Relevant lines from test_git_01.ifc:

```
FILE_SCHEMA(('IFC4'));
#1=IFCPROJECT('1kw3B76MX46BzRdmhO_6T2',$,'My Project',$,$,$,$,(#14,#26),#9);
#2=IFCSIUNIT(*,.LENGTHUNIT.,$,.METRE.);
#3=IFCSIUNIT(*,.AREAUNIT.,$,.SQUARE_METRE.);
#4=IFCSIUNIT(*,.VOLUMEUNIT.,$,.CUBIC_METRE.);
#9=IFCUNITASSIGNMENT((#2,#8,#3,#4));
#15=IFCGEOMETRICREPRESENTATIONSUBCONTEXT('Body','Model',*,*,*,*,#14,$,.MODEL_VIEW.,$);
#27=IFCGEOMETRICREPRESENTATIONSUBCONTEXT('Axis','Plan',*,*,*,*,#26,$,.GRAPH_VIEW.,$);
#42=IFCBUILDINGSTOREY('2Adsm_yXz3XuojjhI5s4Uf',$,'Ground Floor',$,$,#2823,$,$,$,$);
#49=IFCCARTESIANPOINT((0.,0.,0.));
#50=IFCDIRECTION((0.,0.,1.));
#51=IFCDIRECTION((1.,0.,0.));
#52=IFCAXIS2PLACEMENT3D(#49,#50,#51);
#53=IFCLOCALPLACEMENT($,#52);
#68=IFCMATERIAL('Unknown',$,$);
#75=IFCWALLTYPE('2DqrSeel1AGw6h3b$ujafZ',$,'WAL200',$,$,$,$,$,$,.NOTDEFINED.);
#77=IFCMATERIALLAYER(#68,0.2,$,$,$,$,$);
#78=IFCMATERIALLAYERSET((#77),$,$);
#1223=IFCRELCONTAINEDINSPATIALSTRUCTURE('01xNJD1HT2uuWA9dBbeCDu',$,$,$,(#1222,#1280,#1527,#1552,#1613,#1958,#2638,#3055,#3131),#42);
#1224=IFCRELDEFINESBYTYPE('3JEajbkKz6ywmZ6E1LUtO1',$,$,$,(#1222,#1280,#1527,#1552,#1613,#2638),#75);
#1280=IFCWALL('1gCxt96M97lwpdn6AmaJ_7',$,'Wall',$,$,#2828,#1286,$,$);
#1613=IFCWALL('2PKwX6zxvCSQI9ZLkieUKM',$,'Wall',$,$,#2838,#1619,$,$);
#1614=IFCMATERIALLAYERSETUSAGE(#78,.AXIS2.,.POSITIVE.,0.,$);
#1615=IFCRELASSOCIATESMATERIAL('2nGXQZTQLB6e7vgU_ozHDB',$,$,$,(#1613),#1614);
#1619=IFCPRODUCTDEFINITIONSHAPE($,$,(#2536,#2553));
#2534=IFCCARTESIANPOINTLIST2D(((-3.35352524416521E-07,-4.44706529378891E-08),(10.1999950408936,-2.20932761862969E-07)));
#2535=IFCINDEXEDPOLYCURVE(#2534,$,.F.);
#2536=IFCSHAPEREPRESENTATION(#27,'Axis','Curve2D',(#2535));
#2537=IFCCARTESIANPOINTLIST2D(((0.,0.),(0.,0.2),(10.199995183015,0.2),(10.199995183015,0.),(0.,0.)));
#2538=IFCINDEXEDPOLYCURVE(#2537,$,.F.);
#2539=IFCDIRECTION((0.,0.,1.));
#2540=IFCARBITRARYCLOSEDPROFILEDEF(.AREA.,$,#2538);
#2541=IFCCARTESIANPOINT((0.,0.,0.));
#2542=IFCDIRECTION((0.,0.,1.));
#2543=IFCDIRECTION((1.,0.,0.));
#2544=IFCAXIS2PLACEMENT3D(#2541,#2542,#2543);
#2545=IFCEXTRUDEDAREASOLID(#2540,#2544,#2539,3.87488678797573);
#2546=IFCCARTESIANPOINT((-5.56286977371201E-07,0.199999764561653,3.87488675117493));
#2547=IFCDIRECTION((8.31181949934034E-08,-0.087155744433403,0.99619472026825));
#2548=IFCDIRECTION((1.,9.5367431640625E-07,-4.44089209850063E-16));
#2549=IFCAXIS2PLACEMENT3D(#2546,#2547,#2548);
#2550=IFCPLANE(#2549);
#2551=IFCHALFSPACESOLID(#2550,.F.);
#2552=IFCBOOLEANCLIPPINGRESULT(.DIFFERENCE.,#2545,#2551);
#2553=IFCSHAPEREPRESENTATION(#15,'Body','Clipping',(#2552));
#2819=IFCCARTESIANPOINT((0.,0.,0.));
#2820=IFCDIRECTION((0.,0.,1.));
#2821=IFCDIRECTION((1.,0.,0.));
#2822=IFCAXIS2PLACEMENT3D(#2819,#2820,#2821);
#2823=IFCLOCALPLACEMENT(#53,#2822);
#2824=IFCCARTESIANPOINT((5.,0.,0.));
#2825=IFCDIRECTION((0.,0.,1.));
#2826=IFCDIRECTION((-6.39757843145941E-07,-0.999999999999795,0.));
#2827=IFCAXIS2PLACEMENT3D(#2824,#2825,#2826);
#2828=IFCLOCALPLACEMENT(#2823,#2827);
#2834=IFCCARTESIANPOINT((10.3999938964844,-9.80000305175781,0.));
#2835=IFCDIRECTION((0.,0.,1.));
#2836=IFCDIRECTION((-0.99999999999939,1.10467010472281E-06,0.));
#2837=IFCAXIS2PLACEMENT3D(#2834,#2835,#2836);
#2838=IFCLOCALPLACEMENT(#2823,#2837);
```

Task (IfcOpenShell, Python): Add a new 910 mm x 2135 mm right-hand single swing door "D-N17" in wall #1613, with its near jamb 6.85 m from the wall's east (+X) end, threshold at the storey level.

```python
import numpy as np
import ifcopenshell
import ifcopenshell.api.feature
import ifcopenshell.api.geometry
import ifcopenshell.api.root
import ifcopenshell.api.spatial
import ifcopenshell.geom
import ifcopenshell.util.element
import ifcopenshell.util.placement
import ifcopenshell.util.representation
import ifcopenshell.util.shape
import ifcopenshell.util.unit

model = ifcopenshell.open("test_git_01.ifc")
unit_scale = ifcopenshell.util.unit.calculate_unit_scale(model)
settings = ifcopenshell.geom.settings()


def volume(element):
    """Net volume in cubic metres, openings subtracted."""
    shape = ifcopenshell.geom.create_shape(settings, element)
    return ifcopenshell.util.shape.get_volume(shape.geometry)


wall = model.by_id(1613)
storey = ifcopenshell.util.element.get_container(wall, ifc_class="IfcBuildingStorey")
context = ifcopenshell.util.representation.get_context(model, "Model", "Body", "MODEL_VIEW")
before = volume(wall)

width, height, from_end, sill = 0.91, 2.135, 6.85, 0.0  # metres

# The wall runs along its own X axis, and the end named is its -X end.
wall_shape = ifcopenshell.geom.create_shape(settings, wall)
x, y, z = ifcopenshell.util.shape.get_vertices(wall_shape.geometry).T
start = x.min() + from_end
face, thickness = float(y.min()), float(y.max() - y.min())
wall_matrix = ifcopenshell.util.placement.get_local_placement(wall.ObjectPlacement)
level = ifcopenshell.util.placement.get_local_placement(storey.ObjectPlacement)[2, 3]


def in_wall(x, y):
    """Placement at x, y metres in the wall's axes, at sill height."""
    matrix = wall_matrix.copy()
    matrix[:, 3] = wall_matrix @ np.array([x / unit_scale, y / unit_scale, 0.0, 1.0])
    matrix[2, 3] = level + sill / unit_scale
    return matrix


# Opening: a box that overshoots both wall faces by 50 mm.
opening = ifcopenshell.api.root.create_entity(model, ifc_class="IfcOpeningElement", predefined_type="OPENING")
box = ifcopenshell.api.geometry.add_wall_representation(
    model, context=context, length=width, height=height, thickness=thickness + 0.1
)
ifcopenshell.api.geometry.assign_representation(model, product=opening, representation=box)
ifcopenshell.api.geometry.edit_object_placement(model, product=opening, matrix=in_wall(start, face - 0.05), is_si=False)
ifcopenshell.api.feature.add_feature(model, feature=opening, element=wall)

door = ifcopenshell.api.root.create_entity(model, ifc_class="IfcDoor", name="D-N17", predefined_type="DOOR")
door.OverallWidth, door.OverallHeight = width / unit_scale, height / unit_scale
door.OperationType = "SINGLE_SWING_RIGHT"
body = ifcopenshell.api.geometry.add_door_representation(
    model,
    context=context,
    overall_width=door.OverallWidth,
    overall_height=door.OverallHeight,
    operation_type="SINGLE_SWING_RIGHT",
    lining_properties={"LiningDepth": thickness / unit_scale, "ThresholdDepth": thickness / unit_scale},
)
ifcopenshell.api.geometry.assign_representation(model, product=door, representation=body)
ifcopenshell.api.spatial.assign_container(model, products=[door], relating_structure=storey)
ifcopenshell.api.feature.add_filling(model, opening=opening, element=door)

# The lining spans the wall, so the door starts at the wall face.
ifcopenshell.api.geometry.edit_object_placement(model, product=door, matrix=in_wall(start, face), is_si=False)

after = volume(wall)

print(f"wall volume {before:.3f} -> {after:.3f} m3")

model.write("test_git_01_updated.ifc")
```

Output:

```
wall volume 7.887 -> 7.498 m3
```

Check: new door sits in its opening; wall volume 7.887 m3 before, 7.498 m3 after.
